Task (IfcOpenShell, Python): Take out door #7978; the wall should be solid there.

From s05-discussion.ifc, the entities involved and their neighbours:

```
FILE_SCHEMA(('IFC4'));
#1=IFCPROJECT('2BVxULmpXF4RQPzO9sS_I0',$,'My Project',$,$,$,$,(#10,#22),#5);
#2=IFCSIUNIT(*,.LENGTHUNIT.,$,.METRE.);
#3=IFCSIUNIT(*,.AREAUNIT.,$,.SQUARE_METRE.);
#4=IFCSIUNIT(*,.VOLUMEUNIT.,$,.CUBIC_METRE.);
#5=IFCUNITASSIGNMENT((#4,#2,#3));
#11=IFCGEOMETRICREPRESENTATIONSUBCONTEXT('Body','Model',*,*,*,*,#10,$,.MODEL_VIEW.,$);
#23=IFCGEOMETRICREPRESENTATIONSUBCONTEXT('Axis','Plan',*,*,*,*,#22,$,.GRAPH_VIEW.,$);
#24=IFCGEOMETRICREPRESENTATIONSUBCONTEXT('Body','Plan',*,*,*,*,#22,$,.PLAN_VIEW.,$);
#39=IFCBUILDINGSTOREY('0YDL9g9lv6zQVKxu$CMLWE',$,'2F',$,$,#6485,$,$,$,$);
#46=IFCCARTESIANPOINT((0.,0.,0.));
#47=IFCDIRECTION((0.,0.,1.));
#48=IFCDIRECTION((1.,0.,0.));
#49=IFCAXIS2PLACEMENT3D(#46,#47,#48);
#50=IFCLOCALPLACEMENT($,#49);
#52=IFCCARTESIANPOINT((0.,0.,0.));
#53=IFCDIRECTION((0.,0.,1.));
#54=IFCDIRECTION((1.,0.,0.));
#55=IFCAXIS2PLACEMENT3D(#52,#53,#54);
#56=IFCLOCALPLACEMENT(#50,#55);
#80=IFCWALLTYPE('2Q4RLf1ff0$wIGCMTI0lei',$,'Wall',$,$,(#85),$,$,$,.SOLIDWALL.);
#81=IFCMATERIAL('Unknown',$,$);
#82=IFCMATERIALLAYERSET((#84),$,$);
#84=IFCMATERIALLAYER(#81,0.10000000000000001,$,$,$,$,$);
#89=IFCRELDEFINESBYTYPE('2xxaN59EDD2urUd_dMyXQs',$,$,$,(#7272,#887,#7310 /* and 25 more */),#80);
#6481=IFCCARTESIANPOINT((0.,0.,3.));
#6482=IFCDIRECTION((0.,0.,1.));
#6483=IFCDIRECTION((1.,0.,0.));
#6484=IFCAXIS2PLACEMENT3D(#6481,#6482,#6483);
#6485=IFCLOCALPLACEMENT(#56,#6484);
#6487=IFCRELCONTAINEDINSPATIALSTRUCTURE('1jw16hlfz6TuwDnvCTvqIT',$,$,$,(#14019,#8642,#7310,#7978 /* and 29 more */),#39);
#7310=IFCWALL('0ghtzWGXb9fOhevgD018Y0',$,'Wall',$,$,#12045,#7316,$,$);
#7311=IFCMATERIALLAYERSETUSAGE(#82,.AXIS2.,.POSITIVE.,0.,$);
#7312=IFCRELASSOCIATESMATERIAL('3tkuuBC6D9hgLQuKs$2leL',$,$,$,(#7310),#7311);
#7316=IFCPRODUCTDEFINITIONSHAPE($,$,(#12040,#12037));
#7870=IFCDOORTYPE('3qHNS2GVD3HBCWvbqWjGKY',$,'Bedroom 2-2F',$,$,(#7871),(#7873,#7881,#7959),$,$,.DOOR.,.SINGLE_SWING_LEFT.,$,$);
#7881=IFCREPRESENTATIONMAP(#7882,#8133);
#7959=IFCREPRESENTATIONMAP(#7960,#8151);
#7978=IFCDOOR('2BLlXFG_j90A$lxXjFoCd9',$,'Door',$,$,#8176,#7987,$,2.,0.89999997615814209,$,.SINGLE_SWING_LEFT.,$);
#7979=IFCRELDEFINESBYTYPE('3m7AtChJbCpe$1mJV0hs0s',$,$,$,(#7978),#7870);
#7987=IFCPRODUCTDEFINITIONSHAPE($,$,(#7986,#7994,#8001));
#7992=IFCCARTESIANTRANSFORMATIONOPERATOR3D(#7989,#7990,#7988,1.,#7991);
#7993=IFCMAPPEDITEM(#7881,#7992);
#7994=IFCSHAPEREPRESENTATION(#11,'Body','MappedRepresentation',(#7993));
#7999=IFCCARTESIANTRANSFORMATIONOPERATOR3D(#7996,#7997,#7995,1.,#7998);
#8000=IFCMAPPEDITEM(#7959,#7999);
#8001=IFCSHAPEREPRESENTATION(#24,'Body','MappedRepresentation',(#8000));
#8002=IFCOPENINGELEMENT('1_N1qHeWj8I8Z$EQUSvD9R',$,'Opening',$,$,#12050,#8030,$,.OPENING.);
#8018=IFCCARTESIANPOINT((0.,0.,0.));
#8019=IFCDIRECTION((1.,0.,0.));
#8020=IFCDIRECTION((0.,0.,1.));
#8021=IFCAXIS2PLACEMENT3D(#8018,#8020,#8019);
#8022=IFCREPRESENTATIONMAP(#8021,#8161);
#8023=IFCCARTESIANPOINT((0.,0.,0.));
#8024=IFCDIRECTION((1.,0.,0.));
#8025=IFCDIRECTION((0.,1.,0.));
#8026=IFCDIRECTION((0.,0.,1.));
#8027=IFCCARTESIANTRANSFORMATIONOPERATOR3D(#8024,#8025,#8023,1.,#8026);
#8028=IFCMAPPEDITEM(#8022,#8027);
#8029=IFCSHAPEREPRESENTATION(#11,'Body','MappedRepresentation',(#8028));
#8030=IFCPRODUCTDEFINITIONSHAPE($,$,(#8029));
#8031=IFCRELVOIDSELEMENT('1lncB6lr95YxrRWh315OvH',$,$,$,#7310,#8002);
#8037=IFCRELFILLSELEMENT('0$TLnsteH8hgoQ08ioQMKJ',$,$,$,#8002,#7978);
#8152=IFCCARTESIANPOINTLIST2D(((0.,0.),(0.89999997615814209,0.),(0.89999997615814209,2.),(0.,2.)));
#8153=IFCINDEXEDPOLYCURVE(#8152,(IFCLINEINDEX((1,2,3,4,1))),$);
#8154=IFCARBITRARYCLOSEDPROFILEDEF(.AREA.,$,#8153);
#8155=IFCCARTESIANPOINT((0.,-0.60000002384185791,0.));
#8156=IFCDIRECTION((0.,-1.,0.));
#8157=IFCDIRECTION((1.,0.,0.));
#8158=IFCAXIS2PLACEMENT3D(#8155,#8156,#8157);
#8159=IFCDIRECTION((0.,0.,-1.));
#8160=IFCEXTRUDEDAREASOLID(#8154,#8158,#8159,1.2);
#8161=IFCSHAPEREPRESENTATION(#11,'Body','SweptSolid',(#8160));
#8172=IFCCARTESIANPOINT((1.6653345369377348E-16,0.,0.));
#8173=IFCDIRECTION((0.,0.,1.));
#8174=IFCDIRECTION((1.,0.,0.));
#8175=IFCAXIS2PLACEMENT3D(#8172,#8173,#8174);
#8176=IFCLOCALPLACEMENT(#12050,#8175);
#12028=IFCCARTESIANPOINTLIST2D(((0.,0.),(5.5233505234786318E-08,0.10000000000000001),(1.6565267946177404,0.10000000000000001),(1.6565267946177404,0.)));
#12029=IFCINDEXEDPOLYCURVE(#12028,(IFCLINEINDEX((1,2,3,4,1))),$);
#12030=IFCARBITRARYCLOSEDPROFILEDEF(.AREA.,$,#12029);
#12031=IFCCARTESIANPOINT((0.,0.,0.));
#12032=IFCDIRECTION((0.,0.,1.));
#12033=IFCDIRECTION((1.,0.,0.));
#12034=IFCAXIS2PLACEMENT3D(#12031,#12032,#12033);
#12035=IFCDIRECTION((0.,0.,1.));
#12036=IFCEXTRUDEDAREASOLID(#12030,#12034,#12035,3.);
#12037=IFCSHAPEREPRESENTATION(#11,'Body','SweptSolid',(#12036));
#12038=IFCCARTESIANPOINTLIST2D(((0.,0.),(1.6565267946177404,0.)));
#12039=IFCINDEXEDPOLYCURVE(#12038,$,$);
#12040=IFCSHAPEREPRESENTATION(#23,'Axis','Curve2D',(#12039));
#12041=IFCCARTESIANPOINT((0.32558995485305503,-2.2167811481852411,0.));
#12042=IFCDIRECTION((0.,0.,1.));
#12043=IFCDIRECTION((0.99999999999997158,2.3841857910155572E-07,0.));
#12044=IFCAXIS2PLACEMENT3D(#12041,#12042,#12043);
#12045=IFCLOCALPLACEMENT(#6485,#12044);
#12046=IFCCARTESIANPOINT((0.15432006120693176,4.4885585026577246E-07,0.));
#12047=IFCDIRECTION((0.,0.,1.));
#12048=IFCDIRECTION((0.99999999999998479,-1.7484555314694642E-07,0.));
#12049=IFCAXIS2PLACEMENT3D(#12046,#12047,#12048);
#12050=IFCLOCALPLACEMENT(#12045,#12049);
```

```python
import ifcopenshell
import ifcopenshell.api.feature
import ifcopenshell.api.root
import ifcopenshell.geom
import ifcopenshell.util.shape

model = ifcopenshell.open("s05-discussion.ifc")
settings = ifcopenshell.geom.settings()


def volume(element):
    """Net volume in cubic metres, openings subtracted."""
    shape = ifcopenshell.geom.create_shape(settings, element)
    return ifcopenshell.util.shape.get_volume(shape.geometry)


door = model.by_guid("2BLlXFG_j90A$lxXjFoCd9")
opening = door.FillsVoids[0].RelatingOpeningElement
wall = opening.VoidsElements[0].RelatingBuildingElement
before = volume(wall)

ifcopenshell.api.root.remove_product(model, product=door)
ifcopenshell.api.feature.remove_feature(model, feature=opening)

after = volume(wall)

print(f"wall volume {before:.3f} -> {after:.3f} m3")

model.write("s05-discussion_v2.ifc")
```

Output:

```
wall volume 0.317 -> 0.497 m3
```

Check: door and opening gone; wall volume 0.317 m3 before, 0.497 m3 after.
